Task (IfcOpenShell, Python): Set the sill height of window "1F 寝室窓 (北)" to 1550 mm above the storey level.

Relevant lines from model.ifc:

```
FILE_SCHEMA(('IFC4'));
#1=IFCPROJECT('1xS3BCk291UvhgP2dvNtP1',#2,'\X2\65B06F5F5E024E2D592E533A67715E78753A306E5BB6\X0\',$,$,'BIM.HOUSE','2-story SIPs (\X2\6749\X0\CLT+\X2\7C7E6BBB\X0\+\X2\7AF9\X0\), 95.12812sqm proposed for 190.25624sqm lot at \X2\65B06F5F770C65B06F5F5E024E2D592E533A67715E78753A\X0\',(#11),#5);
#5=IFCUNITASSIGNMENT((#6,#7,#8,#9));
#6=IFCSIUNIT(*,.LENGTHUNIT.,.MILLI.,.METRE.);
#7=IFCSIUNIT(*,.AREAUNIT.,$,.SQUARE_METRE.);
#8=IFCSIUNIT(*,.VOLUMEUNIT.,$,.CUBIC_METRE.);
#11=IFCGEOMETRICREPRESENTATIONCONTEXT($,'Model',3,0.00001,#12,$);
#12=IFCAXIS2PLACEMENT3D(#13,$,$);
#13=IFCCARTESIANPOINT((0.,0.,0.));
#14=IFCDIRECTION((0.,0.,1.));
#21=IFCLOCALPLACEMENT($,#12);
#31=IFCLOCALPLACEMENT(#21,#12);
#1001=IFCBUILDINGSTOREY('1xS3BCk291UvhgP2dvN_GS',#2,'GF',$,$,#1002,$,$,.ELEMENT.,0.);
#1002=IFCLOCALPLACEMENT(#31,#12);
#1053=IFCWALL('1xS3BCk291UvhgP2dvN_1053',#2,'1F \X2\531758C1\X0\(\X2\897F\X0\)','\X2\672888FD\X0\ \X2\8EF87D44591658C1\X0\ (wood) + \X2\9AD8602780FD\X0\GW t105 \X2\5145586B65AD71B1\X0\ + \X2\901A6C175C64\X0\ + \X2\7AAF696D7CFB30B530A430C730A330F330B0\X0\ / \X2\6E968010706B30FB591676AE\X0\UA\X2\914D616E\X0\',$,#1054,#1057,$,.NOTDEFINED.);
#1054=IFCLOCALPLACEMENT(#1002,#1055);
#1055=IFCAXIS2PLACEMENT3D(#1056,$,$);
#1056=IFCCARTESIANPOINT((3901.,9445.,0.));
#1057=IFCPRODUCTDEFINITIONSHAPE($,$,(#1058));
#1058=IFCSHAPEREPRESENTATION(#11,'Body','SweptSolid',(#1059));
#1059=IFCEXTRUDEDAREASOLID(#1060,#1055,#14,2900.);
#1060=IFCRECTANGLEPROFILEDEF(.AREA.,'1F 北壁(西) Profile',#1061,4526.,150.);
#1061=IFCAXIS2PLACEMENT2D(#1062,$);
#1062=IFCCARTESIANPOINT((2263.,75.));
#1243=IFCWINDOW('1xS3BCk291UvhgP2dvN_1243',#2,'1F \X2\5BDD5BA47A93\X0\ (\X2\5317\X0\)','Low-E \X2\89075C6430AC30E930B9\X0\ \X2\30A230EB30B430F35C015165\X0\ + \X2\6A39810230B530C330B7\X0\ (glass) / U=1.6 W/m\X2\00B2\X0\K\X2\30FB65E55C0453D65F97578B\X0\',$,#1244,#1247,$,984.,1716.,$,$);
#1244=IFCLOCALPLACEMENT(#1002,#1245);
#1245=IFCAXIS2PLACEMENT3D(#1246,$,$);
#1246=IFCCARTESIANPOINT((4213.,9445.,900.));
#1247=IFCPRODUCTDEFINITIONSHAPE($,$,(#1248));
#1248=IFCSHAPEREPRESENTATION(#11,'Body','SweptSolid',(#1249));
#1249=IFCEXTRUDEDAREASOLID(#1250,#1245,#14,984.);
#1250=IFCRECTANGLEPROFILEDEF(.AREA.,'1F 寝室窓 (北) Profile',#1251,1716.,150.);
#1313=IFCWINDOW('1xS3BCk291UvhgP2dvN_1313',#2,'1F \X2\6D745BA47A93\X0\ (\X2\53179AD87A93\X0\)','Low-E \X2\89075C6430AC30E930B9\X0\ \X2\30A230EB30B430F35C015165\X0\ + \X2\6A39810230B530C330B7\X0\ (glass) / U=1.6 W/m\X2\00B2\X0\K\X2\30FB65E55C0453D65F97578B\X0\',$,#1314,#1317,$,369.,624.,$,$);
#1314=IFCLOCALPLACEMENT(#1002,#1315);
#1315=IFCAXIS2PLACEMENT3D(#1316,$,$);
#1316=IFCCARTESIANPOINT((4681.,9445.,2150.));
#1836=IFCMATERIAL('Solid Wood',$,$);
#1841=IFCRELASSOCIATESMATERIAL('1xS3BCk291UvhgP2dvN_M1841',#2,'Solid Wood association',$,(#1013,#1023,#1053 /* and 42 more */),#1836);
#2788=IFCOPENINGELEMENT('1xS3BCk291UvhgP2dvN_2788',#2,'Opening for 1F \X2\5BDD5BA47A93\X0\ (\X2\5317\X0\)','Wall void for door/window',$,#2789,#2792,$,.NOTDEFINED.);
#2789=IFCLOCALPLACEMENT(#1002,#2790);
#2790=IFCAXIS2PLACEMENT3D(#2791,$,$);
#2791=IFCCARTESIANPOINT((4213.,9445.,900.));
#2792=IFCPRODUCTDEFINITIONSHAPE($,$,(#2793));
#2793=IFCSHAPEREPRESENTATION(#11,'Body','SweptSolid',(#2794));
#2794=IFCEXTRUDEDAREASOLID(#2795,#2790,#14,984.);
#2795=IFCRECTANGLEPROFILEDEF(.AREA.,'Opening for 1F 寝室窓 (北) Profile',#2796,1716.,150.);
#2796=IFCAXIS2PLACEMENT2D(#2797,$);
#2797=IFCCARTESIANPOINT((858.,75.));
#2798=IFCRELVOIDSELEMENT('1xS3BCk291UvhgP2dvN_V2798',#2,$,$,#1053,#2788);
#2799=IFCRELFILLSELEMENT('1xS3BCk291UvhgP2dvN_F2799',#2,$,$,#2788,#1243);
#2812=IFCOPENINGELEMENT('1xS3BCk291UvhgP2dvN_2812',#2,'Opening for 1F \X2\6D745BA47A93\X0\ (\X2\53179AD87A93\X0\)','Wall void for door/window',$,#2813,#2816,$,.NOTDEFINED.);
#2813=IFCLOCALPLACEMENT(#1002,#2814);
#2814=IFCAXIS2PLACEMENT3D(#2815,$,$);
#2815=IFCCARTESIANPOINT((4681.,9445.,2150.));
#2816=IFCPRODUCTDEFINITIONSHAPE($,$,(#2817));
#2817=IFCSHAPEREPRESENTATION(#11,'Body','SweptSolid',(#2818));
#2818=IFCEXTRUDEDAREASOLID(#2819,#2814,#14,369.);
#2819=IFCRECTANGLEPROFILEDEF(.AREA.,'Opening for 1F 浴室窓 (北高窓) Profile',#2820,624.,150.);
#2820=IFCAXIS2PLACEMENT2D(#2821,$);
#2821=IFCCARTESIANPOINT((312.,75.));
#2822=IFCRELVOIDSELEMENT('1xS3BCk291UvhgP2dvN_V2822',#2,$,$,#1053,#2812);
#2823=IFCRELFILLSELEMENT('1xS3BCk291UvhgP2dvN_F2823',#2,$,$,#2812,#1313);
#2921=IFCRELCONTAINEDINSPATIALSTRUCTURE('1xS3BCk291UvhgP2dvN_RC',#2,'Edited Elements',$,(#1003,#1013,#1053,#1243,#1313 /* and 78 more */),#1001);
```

```python
import numpy as np
import ifcopenshell
import ifcopenshell.api.geometry
import ifcopenshell.geom
import ifcopenshell.util.element
import ifcopenshell.util.placement
import ifcopenshell.util.shape
import ifcopenshell.util.unit

model = ifcopenshell.open("model.ifc")
unit_scale = ifcopenshell.util.unit.calculate_unit_scale(model)

window = model.by_id(1243)
opening = window.FillsVoids[0].RelatingOpeningElement
storey = ifcopenshell.util.element.get_container(window, ifc_class="IfcBuildingStorey")
level = ifcopenshell.util.placement.get_local_placement(storey.ObjectPlacement)[2, 3]

# The opening's origin need not be at the sill, so measure its lowest point.
shape = ifcopenshell.geom.create_shape(ifcopenshell.geom.settings(), opening)
bottom = ifcopenshell.util.shape.get_shape_bottom_elevation(shape, shape.geometry) / unit_scale
dz = level + 1.55 / unit_scale - bottom

shift = np.array([0.0, 0.0, dz])
# The window is not placed relative to its opening, so move both.
for product in (opening, window):
    matrix = ifcopenshell.util.placement.get_local_placement(product.ObjectPlacement)
    matrix[:3, 3] += shift
    ifcopenshell.api.geometry.edit_object_placement(model, product=product, matrix=matrix, is_si=False)

print(f"moved by {dz * unit_scale:+.3f} m")

model.write("model_v2.ifc")
```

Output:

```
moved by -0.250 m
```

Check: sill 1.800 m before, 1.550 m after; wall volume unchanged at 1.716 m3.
